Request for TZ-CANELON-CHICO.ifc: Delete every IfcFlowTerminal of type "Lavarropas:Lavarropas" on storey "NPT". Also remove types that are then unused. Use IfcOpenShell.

First a look at what the model holds.

```python
import ifcopenshell
import ifcopenshell.util.element

model = ifcopenshell.open("TZ-CANELON-CHICO.ifc")
print(model.schema)
storey = next(s for s in model.by_type("IfcBuildingStorey") if s.Name == "NPT")
terminals = [e for e in ifcopenshell.util.element.get_decomposition(storey) if e.is_a("IfcFlowTerminal")]
seen = {}
for e in terminals:
    element_type = ifcopenshell.util.element.get_type(e)
    name = element_type.Name if element_type not in (None, e) else None
    seen[name] = seen.get(name, 0) + 1
for name, count in sorted(seen.items(), key=str):
    print(count, "x", name)
```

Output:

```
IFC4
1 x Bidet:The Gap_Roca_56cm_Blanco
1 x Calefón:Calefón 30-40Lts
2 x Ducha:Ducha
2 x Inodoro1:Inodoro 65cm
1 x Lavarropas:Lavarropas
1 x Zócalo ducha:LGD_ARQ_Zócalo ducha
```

```python
import ifcopenshell
import ifcopenshell.api.root
import ifcopenshell.util.element

model = ifcopenshell.open("TZ-CANELON-CHICO.ifc")

storey = next(s for s in model.by_type("IfcBuildingStorey") if s.Name == "NPT")
terminals = [e for e in ifcopenshell.util.element.get_decomposition(storey) if e.is_a("IfcFlowTerminal")]
targets = [e for e in terminals if (t := ifcopenshell.util.element.get_type(e)) not in (None, e) and t.Name == "Lavarropas:Lavarropas"]
types = {ifcopenshell.util.element.get_type(e) for e in targets} - {None, *targets}

for e in targets:
    ifcopenshell.api.root.remove_product(model, product=e)
print(len(targets), "removed")

unused = [t for t in types if not ifcopenshell.util.element.get_types(t)]
for t in unused:
    ifcopenshell.api.root.remove_product(model, product=t)
print(len(unused), "unused types removed")

model.write("TZ-CANELON-CHICO-out.ifc")
```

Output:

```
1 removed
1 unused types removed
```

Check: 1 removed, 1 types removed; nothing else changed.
